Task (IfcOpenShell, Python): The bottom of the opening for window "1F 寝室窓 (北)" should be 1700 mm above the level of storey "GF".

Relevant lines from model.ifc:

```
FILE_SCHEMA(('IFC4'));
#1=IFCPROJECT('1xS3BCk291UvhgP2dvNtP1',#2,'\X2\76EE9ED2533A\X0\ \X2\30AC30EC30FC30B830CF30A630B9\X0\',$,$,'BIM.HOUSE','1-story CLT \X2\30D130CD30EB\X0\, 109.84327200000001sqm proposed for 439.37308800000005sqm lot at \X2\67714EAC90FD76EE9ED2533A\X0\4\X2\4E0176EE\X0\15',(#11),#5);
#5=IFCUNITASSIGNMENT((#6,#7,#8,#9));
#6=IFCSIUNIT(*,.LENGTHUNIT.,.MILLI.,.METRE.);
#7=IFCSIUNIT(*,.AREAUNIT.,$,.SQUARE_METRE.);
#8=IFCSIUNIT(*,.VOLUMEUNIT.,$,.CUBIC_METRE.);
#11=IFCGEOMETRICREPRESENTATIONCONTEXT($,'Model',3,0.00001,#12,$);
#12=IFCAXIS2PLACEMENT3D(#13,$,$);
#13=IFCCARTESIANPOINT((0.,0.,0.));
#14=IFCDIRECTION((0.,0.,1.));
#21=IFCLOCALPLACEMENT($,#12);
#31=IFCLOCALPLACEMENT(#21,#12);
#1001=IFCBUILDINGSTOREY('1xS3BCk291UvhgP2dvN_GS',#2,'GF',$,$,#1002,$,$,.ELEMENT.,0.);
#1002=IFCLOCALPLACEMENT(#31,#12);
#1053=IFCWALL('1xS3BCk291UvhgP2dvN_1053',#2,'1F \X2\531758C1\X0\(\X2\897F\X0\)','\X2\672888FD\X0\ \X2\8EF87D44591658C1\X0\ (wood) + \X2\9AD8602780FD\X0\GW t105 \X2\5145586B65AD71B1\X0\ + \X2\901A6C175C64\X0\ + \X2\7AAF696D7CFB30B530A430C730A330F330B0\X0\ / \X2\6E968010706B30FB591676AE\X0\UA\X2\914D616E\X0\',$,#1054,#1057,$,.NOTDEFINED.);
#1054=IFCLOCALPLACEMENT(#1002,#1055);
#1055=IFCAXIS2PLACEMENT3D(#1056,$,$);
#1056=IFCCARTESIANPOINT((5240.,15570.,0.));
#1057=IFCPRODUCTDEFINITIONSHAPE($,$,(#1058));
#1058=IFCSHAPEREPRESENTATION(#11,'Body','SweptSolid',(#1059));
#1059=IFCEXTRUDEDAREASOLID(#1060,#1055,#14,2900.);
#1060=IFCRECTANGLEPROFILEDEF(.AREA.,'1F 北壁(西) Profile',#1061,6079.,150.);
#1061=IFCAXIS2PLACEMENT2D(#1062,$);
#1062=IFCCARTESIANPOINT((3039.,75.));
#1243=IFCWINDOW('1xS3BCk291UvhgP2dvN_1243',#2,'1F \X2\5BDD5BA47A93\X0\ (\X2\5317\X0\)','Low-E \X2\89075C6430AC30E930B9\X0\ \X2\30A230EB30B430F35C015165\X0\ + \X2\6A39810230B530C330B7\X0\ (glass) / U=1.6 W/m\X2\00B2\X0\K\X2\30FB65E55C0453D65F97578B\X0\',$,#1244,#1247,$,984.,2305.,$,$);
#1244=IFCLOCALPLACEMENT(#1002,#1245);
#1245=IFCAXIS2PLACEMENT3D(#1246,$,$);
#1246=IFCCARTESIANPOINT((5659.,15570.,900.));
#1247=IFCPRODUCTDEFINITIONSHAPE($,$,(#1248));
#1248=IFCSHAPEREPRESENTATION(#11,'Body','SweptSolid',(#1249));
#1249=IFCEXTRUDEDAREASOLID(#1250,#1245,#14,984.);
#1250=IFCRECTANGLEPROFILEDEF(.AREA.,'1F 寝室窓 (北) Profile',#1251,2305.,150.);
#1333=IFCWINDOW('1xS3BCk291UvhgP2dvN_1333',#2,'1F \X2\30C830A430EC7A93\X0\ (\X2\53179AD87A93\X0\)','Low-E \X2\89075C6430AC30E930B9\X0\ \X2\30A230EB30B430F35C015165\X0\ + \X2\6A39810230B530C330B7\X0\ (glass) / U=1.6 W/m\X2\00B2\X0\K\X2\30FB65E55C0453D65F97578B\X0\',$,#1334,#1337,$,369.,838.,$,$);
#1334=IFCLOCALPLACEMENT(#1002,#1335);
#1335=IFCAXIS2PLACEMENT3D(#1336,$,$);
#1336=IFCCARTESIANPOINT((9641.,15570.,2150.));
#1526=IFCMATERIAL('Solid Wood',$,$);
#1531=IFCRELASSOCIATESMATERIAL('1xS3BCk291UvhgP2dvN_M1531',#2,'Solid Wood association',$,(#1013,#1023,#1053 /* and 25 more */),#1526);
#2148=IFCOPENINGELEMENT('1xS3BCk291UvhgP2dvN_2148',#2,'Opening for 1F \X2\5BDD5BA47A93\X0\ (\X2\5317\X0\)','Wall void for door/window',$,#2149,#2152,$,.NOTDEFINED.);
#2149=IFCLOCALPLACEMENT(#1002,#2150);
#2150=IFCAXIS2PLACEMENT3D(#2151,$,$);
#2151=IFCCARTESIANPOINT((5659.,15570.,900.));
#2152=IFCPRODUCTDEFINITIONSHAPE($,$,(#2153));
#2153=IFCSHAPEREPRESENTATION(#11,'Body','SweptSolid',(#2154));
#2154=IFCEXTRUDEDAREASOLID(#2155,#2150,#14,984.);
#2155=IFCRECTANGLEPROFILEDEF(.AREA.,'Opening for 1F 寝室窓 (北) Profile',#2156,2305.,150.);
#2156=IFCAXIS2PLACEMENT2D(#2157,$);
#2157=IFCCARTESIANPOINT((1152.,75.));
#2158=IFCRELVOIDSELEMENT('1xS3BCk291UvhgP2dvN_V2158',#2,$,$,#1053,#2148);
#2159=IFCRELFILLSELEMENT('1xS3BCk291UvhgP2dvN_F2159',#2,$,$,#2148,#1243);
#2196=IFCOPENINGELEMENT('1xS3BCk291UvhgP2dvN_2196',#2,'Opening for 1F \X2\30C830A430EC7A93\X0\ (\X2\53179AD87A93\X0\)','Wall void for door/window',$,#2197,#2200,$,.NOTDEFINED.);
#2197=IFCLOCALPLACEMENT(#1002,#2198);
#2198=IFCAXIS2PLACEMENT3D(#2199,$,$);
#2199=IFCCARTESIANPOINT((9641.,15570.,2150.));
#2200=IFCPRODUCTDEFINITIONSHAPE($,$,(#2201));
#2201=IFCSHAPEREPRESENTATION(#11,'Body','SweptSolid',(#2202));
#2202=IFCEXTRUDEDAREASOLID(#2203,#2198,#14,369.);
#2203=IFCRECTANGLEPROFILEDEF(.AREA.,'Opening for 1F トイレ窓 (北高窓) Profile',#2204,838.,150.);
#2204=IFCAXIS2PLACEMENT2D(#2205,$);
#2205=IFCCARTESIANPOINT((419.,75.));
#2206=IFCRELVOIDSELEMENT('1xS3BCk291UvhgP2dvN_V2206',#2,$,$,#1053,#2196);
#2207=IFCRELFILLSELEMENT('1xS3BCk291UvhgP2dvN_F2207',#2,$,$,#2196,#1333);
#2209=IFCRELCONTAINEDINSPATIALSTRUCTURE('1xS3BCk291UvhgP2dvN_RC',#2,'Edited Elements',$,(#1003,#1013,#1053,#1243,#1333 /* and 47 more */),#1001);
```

```python
import numpy as np
import ifcopenshell
import ifcopenshell.api.geometry
import ifcopenshell.geom
import ifcopenshell.util.element
import ifcopenshell.util.placement
import ifcopenshell.util.shape
import ifcopenshell.util.unit

model = ifcopenshell.open("model.ifc")
unit_scale = ifcopenshell.util.unit.calculate_unit_scale(model)

window = model.by_id(1243)
opening = window.FillsVoids[0].RelatingOpeningElement
storey = ifcopenshell.util.element.get_container(window, ifc_class="IfcBuildingStorey")
level = ifcopenshell.util.placement.get_local_placement(storey.ObjectPlacement)[2, 3]

# The opening's origin need not be at the sill, so measure its lowest point.
shape = ifcopenshell.geom.create_shape(ifcopenshell.geom.settings(), opening)
bottom = ifcopenshell.util.shape.get_shape_bottom_elevation(shape, shape.geometry) / unit_scale
dz = level + 1.7 / unit_scale - bottom

shift = np.array([0.0, 0.0, dz])
# The window is not placed relative to its opening, so move both.
for product in (opening, window):
    matrix = ifcopenshell.util.placement.get_local_placement(product.ObjectPlacement)
    matrix[:3, 3] += shift
    ifcopenshell.api.geometry.edit_object_placement(model, product=product, matrix=matrix, is_si=False)

print(f"moved by {dz * unit_scale:+.3f} m")

model.write("model_v2.ifc")
```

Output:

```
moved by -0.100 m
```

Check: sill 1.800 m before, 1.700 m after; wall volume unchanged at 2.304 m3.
